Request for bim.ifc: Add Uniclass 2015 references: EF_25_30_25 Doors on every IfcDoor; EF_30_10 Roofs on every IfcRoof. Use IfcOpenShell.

First a look at what the model holds.

```python
import ifcopenshell

model = ifcopenshell.open("bim.ifc")
print(model.schema)
print("classifications:", [c.Name for c in model.by_type("IfcClassification")])
for ifc_class in ("IfcDoor", "IfcRoof", "IfcStair", "IfcWall", "IfcWindow"):
    print(ifc_class, len(model.by_type(ifc_class)))
```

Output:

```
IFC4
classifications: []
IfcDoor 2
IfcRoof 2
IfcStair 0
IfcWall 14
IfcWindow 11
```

```python
import ifcopenshell
import ifcopenshell.api.classification

model = ifcopenshell.open("bim.ifc")

system = ifcopenshell.api.classification.add_classification(model, classification="Uniclass 2015")

codes = {
    "IfcDoor": ("EF_25_30_25", "Doors"),
    "IfcRoof": ("EF_30_10", "Roofs"),
}
for ifc_class, (code, name) in codes.items():
    products = model.by_type(ifc_class)
    ifcopenshell.api.classification.add_reference(
        model, products=products, classification=system, identification=code, name=name
    )
    print(code, len(products))

model.write("bim_updated.ifc")
```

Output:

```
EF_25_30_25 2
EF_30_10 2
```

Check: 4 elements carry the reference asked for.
